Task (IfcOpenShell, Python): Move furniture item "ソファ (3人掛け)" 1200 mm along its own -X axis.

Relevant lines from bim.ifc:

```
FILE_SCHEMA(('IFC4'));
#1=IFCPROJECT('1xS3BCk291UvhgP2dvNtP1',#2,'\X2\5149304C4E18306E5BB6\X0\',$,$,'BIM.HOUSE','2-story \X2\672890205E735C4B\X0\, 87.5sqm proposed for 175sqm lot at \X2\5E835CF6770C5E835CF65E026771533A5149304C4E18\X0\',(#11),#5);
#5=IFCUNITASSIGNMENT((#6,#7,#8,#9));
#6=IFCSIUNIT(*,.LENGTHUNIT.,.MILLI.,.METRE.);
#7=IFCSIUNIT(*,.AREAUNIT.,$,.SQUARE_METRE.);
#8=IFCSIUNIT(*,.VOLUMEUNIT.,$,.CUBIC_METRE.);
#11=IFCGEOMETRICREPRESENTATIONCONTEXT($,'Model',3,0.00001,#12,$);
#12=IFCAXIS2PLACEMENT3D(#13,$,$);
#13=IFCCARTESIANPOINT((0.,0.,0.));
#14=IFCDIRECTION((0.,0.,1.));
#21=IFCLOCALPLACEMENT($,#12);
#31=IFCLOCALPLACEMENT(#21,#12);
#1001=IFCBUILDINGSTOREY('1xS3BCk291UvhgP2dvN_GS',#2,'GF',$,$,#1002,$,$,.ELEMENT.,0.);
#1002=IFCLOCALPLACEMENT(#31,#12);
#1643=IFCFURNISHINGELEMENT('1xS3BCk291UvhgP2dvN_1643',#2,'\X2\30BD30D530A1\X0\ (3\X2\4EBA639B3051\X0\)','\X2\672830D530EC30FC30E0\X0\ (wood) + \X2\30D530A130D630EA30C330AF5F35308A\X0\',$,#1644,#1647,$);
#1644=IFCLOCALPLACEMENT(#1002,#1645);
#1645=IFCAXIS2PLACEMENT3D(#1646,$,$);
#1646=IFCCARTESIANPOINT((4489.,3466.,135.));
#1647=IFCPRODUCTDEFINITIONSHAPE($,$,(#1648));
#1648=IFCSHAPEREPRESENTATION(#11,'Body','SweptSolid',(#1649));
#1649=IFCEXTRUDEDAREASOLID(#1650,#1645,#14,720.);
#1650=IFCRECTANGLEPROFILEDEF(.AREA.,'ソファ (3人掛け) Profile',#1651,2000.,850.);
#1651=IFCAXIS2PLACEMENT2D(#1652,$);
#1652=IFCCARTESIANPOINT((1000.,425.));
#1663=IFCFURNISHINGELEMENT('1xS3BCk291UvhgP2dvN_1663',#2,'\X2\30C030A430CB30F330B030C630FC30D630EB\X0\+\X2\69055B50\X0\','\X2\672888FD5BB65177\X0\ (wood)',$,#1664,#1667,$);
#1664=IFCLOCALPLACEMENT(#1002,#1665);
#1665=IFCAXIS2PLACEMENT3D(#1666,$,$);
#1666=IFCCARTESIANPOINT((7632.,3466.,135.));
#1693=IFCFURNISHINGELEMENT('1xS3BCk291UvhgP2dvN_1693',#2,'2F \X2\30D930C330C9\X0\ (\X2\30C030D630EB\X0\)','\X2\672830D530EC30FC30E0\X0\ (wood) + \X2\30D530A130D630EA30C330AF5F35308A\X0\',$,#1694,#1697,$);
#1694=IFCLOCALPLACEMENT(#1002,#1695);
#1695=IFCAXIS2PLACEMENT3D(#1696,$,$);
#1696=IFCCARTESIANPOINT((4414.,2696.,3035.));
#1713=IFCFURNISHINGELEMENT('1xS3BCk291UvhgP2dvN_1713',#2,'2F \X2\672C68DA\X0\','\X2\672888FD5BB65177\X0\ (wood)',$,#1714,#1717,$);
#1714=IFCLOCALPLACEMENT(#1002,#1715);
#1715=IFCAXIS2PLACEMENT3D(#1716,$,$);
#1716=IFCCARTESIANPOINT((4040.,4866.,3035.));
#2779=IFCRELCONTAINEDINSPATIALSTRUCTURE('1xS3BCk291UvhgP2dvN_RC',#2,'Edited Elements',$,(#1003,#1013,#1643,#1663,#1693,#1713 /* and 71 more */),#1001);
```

```python
import ifcopenshell
import ifcopenshell.api.geometry
import ifcopenshell.util.placement

model = ifcopenshell.open("bim.ifc")

item = model.by_guid("1xS3BCk291UvhgP2dvN_1643")
matrix = ifcopenshell.util.placement.get_local_placement(item.ObjectPlacement)
matrix[:3, 3] -= matrix[:3, 0] * 1200.0
ifcopenshell.api.geometry.edit_object_placement(model, product=item, matrix=matrix, is_si=False)

print(ifcopenshell.util.placement.get_local_placement(item.ObjectPlacement).round(3) + 0.0)

model.write("bim_v2.ifc")
```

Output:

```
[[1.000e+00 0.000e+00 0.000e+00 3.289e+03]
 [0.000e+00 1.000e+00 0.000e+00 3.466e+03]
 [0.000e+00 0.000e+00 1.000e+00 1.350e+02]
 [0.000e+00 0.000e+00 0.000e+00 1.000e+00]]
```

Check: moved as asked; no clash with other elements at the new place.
